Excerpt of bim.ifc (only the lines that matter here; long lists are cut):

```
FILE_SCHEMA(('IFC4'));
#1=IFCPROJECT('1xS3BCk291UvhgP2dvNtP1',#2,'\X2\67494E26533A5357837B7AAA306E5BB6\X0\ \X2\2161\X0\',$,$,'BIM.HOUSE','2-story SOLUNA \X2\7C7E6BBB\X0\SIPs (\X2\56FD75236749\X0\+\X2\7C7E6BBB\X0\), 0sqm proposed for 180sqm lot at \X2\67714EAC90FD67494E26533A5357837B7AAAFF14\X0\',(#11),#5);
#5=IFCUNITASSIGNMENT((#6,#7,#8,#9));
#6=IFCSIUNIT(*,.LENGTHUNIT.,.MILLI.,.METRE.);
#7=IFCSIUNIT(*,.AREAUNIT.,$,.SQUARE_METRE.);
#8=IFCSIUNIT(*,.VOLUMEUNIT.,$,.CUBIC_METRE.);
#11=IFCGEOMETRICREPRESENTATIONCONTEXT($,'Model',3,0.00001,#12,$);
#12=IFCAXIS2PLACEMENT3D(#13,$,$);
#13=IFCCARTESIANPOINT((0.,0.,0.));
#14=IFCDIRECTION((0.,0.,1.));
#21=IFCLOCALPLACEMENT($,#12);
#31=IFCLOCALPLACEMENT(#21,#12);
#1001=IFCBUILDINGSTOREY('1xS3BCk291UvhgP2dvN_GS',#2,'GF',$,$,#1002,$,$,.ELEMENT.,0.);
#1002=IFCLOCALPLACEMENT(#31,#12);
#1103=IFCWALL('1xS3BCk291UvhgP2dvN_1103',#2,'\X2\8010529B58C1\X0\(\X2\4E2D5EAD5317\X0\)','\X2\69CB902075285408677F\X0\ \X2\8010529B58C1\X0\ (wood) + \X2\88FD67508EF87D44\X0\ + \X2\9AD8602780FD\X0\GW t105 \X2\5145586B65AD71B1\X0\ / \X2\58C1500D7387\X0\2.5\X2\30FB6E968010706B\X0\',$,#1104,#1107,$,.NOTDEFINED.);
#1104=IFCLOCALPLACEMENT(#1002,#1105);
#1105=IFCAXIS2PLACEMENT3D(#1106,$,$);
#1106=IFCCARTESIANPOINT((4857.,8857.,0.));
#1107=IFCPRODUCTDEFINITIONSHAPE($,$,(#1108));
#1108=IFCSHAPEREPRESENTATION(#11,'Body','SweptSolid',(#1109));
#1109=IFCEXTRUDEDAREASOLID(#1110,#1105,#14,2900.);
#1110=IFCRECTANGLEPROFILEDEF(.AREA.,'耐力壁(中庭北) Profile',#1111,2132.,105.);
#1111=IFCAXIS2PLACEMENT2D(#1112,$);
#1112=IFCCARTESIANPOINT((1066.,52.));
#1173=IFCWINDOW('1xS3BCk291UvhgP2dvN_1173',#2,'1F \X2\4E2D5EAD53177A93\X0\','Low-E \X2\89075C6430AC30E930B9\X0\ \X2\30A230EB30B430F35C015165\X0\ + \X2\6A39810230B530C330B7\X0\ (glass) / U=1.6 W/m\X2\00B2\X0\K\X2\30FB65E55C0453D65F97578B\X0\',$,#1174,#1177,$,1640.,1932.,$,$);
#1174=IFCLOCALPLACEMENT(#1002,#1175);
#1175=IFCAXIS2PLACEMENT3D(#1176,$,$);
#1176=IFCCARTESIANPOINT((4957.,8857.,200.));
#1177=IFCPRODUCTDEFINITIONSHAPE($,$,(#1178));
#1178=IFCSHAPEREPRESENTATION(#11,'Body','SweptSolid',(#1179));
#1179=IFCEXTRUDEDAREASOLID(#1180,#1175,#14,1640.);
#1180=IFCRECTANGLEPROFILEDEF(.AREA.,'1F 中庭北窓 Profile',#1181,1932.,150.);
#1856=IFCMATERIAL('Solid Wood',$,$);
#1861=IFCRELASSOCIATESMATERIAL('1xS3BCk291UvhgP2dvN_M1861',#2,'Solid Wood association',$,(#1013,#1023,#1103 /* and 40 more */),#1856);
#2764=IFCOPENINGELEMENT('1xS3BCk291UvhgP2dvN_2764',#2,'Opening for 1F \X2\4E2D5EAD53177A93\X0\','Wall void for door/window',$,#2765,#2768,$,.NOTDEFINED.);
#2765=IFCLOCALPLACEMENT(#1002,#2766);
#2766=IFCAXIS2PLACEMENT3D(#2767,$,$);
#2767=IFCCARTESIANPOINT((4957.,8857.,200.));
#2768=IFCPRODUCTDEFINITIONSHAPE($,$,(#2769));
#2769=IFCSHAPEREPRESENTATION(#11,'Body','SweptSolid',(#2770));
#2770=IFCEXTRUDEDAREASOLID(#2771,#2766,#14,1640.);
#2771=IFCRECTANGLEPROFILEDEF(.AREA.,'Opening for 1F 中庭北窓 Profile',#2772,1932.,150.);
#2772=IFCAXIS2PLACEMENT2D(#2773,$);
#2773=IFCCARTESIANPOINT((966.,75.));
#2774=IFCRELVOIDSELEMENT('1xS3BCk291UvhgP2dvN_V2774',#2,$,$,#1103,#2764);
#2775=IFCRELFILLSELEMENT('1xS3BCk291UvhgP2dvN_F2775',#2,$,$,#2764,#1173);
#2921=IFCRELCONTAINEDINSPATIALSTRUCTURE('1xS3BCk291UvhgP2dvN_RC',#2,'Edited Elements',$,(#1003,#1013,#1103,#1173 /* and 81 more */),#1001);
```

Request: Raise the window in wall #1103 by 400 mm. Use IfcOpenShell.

```python
import numpy as np
import ifcopenshell
import ifcopenshell.api.geometry
import ifcopenshell.util.placement
import ifcopenshell.util.unit

model = ifcopenshell.open("bim.ifc")
unit_scale = ifcopenshell.util.unit.calculate_unit_scale(model)

window = model.by_id(1173)
opening = window.FillsVoids[0].RelatingOpeningElement
dz = 400.0

shift = np.array([0.0, 0.0, dz])
# The window is not placed relative to its opening, so move both.
for product in (opening, window):
    matrix = ifcopenshell.util.placement.get_local_placement(product.ObjectPlacement)
    matrix[:3, 3] += shift
    ifcopenshell.api.geometry.edit_object_placement(model, product=product, matrix=matrix, is_si=False)

print(f"moved by {dz * unit_scale:+.3f} m")

model.write("bim_rev.ifc")
```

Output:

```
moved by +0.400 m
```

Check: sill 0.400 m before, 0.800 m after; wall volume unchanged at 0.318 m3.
